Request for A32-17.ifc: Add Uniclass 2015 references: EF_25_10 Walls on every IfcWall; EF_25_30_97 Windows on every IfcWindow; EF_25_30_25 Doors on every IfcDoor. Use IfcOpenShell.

First a look at what the model holds.

```python
import ifcopenshell

model = ifcopenshell.open("A32-17.ifc")
print(model.schema)
print("classifications:", [c.Name for c in model.by_type("IfcClassification")])
for ifc_class in ("IfcDoor", "IfcRoof", "IfcStair", "IfcWall", "IfcWindow"):
    print(ifc_class, len(model.by_type(ifc_class)))
```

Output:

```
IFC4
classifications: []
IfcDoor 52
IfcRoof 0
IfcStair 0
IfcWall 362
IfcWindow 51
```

```python
import ifcopenshell
import ifcopenshell.api.classification

model = ifcopenshell.open("A32-17.ifc")

system = ifcopenshell.api.classification.add_classification(model, classification="Uniclass 2015")

codes = {
    "IfcWall": ("EF_25_10", "Walls"),
    "IfcWindow": ("EF_25_30_97", "Windows"),
    "IfcDoor": ("EF_25_30_25", "Doors"),
}
for ifc_class, (code, name) in codes.items():
    products = model.by_type(ifc_class)
    ifcopenshell.api.classification.add_reference(
        model, products=products, classification=system, identification=code, name=name
    )
    print(code, len(products))

model.write("A32-17_rev.ifc")
```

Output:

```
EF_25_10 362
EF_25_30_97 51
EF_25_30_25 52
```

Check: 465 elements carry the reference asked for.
